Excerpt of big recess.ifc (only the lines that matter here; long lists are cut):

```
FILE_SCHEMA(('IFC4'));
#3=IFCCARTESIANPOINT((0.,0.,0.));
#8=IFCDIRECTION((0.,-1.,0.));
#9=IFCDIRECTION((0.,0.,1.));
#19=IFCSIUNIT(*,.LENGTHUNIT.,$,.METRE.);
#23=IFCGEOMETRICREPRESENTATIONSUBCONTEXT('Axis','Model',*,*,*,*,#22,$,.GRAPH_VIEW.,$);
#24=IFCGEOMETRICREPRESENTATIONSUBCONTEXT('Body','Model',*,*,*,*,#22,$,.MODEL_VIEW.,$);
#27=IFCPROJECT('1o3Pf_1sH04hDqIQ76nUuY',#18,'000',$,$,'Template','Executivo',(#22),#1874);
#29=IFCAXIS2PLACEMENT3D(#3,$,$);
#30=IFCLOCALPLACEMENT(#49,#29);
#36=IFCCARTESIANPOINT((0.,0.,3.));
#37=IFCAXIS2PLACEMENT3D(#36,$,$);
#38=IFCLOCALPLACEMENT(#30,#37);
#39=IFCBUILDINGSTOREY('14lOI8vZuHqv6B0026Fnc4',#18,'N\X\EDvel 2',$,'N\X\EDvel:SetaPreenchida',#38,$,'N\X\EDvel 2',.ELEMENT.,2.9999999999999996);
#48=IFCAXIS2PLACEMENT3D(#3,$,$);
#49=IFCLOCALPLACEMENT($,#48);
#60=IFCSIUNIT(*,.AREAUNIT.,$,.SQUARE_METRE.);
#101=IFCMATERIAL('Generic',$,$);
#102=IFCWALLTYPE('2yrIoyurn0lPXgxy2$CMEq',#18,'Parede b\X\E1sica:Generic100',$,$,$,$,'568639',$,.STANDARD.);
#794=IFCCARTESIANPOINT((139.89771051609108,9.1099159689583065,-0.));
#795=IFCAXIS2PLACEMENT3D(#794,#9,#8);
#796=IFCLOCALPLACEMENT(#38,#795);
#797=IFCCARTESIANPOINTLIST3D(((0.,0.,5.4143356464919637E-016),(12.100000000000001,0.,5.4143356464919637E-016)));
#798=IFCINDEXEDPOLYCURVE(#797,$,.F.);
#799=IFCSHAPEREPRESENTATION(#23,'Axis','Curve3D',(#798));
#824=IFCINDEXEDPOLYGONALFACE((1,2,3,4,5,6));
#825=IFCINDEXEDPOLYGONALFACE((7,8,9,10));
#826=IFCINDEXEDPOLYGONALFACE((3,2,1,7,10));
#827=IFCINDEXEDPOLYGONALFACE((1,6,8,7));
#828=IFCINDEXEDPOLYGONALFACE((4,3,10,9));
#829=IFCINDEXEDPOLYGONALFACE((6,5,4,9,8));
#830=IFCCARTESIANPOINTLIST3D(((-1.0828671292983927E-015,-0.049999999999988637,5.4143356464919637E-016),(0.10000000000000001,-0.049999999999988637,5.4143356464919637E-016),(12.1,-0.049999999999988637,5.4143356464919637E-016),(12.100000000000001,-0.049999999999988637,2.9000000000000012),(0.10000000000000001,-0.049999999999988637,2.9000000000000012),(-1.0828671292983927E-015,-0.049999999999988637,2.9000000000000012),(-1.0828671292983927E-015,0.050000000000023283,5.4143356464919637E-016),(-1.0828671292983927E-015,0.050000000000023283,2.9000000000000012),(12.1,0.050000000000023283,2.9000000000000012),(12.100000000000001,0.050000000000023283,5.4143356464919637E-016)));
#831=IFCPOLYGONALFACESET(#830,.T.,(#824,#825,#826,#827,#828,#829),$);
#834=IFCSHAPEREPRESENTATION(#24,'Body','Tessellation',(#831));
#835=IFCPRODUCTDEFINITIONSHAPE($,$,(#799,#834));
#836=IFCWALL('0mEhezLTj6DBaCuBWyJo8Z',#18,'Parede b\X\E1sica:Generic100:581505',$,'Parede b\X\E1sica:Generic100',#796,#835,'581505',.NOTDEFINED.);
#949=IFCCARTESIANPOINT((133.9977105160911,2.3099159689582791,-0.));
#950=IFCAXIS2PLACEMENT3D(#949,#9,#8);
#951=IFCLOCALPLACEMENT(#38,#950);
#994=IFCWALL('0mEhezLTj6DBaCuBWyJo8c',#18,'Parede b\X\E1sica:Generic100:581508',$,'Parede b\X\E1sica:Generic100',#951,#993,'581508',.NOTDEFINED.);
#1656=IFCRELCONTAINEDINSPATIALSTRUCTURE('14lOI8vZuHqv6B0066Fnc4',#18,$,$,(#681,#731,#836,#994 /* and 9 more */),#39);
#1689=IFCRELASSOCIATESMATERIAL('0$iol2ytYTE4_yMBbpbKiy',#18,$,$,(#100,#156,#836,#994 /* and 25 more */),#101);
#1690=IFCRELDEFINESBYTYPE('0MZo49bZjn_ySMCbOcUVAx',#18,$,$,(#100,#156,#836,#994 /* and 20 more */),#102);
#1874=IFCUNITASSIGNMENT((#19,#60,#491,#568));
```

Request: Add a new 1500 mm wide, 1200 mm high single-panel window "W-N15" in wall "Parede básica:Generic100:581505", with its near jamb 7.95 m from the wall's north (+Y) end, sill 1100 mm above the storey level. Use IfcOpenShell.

```python
import numpy as np
import ifcopenshell
import ifcopenshell.api.feature
import ifcopenshell.api.geometry
import ifcopenshell.api.root
import ifcopenshell.api.spatial
import ifcopenshell.geom
import ifcopenshell.util.element
import ifcopenshell.util.placement
import ifcopenshell.util.representation
import ifcopenshell.util.shape
import ifcopenshell.util.unit

model = ifcopenshell.open("big recess.ifc")
unit_scale = ifcopenshell.util.unit.calculate_unit_scale(model)
settings = ifcopenshell.geom.settings()


def volume(element):
    """Net volume in cubic metres, openings subtracted."""
    shape = ifcopenshell.geom.create_shape(settings, element)
    return ifcopenshell.util.shape.get_volume(shape.geometry)


wall = model.by_guid("0mEhezLTj6DBaCuBWyJo8Z")
storey = ifcopenshell.util.element.get_container(wall, ifc_class="IfcBuildingStorey")
context = ifcopenshell.util.representation.get_context(model, "Model", "Body", "MODEL_VIEW")
before = volume(wall)

width, height, from_end, sill = 1.5, 1.2, 7.95, 1.1  # metres

# The wall runs along its own X axis, and the end named is its -X end.
wall_shape = ifcopenshell.geom.create_shape(settings, wall)
x, y, z = ifcopenshell.util.shape.get_vertices(wall_shape.geometry).T
start = x.min() + from_end
face, thickness = float(y.min()), float(y.max() - y.min())
wall_matrix = ifcopenshell.util.placement.get_local_placement(wall.ObjectPlacement)
level = ifcopenshell.util.placement.get_local_placement(storey.ObjectPlacement)[2, 3]


def in_wall(x, y):
    """Placement at x, y metres in the wall's axes, at sill height."""
    matrix = wall_matrix.copy()
    matrix[:, 3] = wall_matrix @ np.array([x / unit_scale, y / unit_scale, 0.0, 1.0])
    matrix[2, 3] = level + sill / unit_scale
    return matrix


# Opening: a box that overshoots both wall faces by 50 mm.
opening = ifcopenshell.api.root.create_entity(model, ifc_class="IfcOpeningElement", predefined_type="OPENING")
box = ifcopenshell.api.geometry.add_wall_representation(
    model, context=context, length=width, height=height, thickness=thickness + 0.1
)
ifcopenshell.api.geometry.assign_representation(model, product=opening, representation=box)
ifcopenshell.api.geometry.edit_object_placement(model, product=opening, matrix=in_wall(start, face - 0.05), is_si=False)
ifcopenshell.api.feature.add_feature(model, feature=opening, element=wall)

window = ifcopenshell.api.root.create_entity(model, ifc_class="IfcWindow", name="W-N15", predefined_type="WINDOW")
window.OverallWidth, window.OverallHeight = width / unit_scale, height / unit_scale
window.PartitioningType = "SINGLE_PANEL"
body = ifcopenshell.api.geometry.add_window_representation(
    model,
    context=context,
    overall_width=window.OverallWidth,
    overall_height=window.OverallHeight,
    partition_type="SINGLE_PANEL",
)
ifcopenshell.api.geometry.assign_representation(model, product=window, representation=body)
ifcopenshell.api.spatial.assign_container(model, products=[window], relating_structure=storey)
ifcopenshell.api.feature.add_filling(model, opening=opening, element=window)

# Centre the window in the wall's thickness.
ifcopenshell.api.geometry.edit_object_placement(model, product=window, matrix=in_wall(start, face), is_si=False)
window_shape = ifcopenshell.geom.create_shape(settings, window)
depth = ifcopenshell.util.shape.get_vertices(window_shape.geometry)[:, 1]
offset = face + thickness / 2 - (depth.min() + depth.max()) / 2
ifcopenshell.api.geometry.edit_object_placement(model, product=window, matrix=in_wall(start, offset), is_si=False)

after = volume(wall)

print(f"wall volume {before:.3f} -> {after:.3f} m3")

model.write("big recess_rev.ifc")
```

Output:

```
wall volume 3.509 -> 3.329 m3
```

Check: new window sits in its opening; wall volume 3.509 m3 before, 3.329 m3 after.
